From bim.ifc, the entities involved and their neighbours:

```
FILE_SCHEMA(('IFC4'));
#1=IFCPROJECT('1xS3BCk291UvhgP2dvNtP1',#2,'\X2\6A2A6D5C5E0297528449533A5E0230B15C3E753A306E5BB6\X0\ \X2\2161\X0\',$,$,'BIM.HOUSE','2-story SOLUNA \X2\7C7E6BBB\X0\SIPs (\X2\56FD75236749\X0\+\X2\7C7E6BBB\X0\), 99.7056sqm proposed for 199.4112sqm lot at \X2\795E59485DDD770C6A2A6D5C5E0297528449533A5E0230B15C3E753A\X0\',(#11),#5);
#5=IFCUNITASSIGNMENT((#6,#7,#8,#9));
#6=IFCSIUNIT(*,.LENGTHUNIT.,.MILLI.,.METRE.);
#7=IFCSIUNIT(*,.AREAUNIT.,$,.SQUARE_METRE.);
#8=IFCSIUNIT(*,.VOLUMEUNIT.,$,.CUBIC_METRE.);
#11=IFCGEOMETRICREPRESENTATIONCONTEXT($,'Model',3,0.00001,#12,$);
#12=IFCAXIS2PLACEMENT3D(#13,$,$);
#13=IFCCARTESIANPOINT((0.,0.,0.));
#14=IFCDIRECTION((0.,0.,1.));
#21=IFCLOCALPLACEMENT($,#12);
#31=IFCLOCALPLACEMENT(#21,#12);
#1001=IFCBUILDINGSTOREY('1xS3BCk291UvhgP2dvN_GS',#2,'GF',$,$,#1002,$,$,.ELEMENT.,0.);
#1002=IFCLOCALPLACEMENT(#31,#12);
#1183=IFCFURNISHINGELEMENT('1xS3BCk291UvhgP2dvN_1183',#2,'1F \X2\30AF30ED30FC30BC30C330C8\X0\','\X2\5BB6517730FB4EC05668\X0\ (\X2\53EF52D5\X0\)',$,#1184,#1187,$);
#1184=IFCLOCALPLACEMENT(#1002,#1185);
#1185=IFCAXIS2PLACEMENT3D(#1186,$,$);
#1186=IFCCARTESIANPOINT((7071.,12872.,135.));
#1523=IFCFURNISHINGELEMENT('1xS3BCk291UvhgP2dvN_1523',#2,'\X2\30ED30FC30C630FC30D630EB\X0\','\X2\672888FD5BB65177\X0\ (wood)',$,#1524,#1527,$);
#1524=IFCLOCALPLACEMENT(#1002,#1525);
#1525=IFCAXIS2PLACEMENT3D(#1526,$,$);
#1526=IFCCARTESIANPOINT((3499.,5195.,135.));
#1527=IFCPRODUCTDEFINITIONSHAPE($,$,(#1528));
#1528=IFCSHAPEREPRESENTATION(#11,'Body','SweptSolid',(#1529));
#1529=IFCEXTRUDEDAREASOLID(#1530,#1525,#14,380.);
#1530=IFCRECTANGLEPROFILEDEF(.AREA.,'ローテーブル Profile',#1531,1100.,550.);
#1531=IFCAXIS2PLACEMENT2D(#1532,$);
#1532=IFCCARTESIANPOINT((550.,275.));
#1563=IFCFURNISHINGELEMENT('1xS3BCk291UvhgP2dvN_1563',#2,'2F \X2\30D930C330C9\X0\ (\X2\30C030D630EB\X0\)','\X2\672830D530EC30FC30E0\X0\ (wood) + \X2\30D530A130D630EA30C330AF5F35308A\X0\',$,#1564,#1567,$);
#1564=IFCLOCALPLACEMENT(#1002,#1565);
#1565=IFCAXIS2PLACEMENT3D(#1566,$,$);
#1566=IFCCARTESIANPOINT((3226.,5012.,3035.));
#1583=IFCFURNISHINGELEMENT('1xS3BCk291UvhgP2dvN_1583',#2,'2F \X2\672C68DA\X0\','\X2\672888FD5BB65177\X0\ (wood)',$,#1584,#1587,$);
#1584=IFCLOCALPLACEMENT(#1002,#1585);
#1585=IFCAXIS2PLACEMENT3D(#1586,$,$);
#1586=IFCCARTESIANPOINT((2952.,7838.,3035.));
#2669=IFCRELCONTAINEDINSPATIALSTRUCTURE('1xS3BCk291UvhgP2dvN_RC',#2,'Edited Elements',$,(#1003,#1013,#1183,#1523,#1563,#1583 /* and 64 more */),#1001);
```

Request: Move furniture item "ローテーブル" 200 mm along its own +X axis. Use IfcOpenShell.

```python
import ifcopenshell
import ifcopenshell.api.geometry
import ifcopenshell.util.placement
import ifcopenshell.util.unit

model = ifcopenshell.open("bim.ifc")
unit_scale = ifcopenshell.util.unit.calculate_unit_scale(model)

item = model.by_id(1523)
matrix = ifcopenshell.util.placement.get_local_placement(item.ObjectPlacement)
matrix[:3, 3] += matrix[:3, 0] * 0.2 / unit_scale
ifcopenshell.api.geometry.edit_object_placement(model, product=item, matrix=matrix, is_si=False)

print(ifcopenshell.util.placement.get_local_placement(item.ObjectPlacement).round(3) + 0.0)

model.write("bim-out.ifc")
```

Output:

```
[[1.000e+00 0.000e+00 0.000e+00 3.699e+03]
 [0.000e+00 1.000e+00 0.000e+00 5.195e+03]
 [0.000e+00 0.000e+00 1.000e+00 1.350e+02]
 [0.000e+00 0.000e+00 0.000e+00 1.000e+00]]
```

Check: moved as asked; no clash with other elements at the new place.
